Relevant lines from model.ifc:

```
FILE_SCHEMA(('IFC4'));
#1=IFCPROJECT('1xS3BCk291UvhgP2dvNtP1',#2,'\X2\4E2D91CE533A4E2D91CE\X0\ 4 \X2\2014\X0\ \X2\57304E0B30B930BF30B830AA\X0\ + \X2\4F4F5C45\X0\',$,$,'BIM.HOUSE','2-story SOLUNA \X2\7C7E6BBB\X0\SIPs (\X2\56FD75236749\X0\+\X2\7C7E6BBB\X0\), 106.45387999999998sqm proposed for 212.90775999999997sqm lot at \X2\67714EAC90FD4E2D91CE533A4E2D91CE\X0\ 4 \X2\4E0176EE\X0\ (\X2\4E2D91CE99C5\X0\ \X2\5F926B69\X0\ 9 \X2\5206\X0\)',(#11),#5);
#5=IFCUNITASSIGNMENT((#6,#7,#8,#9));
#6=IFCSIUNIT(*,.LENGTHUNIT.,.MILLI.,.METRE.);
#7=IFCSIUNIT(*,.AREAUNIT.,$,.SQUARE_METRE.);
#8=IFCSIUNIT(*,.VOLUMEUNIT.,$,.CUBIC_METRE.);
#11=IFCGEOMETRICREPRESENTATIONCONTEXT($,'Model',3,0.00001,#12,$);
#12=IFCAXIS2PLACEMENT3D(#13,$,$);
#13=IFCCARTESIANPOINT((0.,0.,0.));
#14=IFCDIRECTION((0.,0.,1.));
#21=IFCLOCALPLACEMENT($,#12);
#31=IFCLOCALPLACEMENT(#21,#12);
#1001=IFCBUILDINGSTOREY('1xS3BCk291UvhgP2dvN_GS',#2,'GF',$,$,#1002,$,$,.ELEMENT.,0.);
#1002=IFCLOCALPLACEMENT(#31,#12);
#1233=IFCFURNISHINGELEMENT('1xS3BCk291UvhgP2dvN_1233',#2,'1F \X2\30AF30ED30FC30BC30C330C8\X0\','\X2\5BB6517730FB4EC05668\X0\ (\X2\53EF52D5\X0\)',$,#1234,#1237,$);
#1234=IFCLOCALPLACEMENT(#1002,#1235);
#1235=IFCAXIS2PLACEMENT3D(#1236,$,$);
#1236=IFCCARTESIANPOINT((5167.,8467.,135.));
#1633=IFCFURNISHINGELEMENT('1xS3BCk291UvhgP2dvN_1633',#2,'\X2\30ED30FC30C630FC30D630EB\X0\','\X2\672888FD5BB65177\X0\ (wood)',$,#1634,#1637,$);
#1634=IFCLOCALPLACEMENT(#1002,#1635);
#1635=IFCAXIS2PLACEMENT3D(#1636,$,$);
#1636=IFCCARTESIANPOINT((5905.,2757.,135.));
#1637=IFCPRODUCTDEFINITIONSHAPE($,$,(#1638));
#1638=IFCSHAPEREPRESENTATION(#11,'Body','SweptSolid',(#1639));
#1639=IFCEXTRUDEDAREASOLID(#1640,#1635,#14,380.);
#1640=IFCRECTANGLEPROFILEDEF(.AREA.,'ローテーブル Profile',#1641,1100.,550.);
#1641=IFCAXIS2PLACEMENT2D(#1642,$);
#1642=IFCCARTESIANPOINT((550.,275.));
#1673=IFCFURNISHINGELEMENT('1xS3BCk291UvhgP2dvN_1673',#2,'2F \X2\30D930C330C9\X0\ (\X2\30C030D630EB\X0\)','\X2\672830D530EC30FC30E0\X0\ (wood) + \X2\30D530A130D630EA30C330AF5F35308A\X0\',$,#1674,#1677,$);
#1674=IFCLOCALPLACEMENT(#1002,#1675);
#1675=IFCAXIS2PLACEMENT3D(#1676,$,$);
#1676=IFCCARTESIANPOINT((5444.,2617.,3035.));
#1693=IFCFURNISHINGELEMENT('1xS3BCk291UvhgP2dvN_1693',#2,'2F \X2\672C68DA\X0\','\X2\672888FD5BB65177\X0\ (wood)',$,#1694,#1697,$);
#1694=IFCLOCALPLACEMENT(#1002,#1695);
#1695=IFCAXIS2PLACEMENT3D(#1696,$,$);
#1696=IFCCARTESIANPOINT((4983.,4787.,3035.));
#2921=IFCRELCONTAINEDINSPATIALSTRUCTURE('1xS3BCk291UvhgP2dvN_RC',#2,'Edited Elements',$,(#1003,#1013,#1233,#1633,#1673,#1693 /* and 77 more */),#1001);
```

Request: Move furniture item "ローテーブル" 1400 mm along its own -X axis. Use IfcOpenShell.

```python
import ifcopenshell
import ifcopenshell.api.geometry
import ifcopenshell.util.placement

model = ifcopenshell.open("model.ifc")

item = model.by_guid("1xS3BCk291UvhgP2dvN_1633")
matrix = ifcopenshell.util.placement.get_local_placement(item.ObjectPlacement)
matrix[:3, 3] -= matrix[:3, 0] * 1400.0
ifcopenshell.api.geometry.edit_object_placement(model, product=item, matrix=matrix, is_si=False)

print(ifcopenshell.util.placement.get_local_placement(item.ObjectPlacement).round(3) + 0.0)

model.write("model_rev.ifc")
```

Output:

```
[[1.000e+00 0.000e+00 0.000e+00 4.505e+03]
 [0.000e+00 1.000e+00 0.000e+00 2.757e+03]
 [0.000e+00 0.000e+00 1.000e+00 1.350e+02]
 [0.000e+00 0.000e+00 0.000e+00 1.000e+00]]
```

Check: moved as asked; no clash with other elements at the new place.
